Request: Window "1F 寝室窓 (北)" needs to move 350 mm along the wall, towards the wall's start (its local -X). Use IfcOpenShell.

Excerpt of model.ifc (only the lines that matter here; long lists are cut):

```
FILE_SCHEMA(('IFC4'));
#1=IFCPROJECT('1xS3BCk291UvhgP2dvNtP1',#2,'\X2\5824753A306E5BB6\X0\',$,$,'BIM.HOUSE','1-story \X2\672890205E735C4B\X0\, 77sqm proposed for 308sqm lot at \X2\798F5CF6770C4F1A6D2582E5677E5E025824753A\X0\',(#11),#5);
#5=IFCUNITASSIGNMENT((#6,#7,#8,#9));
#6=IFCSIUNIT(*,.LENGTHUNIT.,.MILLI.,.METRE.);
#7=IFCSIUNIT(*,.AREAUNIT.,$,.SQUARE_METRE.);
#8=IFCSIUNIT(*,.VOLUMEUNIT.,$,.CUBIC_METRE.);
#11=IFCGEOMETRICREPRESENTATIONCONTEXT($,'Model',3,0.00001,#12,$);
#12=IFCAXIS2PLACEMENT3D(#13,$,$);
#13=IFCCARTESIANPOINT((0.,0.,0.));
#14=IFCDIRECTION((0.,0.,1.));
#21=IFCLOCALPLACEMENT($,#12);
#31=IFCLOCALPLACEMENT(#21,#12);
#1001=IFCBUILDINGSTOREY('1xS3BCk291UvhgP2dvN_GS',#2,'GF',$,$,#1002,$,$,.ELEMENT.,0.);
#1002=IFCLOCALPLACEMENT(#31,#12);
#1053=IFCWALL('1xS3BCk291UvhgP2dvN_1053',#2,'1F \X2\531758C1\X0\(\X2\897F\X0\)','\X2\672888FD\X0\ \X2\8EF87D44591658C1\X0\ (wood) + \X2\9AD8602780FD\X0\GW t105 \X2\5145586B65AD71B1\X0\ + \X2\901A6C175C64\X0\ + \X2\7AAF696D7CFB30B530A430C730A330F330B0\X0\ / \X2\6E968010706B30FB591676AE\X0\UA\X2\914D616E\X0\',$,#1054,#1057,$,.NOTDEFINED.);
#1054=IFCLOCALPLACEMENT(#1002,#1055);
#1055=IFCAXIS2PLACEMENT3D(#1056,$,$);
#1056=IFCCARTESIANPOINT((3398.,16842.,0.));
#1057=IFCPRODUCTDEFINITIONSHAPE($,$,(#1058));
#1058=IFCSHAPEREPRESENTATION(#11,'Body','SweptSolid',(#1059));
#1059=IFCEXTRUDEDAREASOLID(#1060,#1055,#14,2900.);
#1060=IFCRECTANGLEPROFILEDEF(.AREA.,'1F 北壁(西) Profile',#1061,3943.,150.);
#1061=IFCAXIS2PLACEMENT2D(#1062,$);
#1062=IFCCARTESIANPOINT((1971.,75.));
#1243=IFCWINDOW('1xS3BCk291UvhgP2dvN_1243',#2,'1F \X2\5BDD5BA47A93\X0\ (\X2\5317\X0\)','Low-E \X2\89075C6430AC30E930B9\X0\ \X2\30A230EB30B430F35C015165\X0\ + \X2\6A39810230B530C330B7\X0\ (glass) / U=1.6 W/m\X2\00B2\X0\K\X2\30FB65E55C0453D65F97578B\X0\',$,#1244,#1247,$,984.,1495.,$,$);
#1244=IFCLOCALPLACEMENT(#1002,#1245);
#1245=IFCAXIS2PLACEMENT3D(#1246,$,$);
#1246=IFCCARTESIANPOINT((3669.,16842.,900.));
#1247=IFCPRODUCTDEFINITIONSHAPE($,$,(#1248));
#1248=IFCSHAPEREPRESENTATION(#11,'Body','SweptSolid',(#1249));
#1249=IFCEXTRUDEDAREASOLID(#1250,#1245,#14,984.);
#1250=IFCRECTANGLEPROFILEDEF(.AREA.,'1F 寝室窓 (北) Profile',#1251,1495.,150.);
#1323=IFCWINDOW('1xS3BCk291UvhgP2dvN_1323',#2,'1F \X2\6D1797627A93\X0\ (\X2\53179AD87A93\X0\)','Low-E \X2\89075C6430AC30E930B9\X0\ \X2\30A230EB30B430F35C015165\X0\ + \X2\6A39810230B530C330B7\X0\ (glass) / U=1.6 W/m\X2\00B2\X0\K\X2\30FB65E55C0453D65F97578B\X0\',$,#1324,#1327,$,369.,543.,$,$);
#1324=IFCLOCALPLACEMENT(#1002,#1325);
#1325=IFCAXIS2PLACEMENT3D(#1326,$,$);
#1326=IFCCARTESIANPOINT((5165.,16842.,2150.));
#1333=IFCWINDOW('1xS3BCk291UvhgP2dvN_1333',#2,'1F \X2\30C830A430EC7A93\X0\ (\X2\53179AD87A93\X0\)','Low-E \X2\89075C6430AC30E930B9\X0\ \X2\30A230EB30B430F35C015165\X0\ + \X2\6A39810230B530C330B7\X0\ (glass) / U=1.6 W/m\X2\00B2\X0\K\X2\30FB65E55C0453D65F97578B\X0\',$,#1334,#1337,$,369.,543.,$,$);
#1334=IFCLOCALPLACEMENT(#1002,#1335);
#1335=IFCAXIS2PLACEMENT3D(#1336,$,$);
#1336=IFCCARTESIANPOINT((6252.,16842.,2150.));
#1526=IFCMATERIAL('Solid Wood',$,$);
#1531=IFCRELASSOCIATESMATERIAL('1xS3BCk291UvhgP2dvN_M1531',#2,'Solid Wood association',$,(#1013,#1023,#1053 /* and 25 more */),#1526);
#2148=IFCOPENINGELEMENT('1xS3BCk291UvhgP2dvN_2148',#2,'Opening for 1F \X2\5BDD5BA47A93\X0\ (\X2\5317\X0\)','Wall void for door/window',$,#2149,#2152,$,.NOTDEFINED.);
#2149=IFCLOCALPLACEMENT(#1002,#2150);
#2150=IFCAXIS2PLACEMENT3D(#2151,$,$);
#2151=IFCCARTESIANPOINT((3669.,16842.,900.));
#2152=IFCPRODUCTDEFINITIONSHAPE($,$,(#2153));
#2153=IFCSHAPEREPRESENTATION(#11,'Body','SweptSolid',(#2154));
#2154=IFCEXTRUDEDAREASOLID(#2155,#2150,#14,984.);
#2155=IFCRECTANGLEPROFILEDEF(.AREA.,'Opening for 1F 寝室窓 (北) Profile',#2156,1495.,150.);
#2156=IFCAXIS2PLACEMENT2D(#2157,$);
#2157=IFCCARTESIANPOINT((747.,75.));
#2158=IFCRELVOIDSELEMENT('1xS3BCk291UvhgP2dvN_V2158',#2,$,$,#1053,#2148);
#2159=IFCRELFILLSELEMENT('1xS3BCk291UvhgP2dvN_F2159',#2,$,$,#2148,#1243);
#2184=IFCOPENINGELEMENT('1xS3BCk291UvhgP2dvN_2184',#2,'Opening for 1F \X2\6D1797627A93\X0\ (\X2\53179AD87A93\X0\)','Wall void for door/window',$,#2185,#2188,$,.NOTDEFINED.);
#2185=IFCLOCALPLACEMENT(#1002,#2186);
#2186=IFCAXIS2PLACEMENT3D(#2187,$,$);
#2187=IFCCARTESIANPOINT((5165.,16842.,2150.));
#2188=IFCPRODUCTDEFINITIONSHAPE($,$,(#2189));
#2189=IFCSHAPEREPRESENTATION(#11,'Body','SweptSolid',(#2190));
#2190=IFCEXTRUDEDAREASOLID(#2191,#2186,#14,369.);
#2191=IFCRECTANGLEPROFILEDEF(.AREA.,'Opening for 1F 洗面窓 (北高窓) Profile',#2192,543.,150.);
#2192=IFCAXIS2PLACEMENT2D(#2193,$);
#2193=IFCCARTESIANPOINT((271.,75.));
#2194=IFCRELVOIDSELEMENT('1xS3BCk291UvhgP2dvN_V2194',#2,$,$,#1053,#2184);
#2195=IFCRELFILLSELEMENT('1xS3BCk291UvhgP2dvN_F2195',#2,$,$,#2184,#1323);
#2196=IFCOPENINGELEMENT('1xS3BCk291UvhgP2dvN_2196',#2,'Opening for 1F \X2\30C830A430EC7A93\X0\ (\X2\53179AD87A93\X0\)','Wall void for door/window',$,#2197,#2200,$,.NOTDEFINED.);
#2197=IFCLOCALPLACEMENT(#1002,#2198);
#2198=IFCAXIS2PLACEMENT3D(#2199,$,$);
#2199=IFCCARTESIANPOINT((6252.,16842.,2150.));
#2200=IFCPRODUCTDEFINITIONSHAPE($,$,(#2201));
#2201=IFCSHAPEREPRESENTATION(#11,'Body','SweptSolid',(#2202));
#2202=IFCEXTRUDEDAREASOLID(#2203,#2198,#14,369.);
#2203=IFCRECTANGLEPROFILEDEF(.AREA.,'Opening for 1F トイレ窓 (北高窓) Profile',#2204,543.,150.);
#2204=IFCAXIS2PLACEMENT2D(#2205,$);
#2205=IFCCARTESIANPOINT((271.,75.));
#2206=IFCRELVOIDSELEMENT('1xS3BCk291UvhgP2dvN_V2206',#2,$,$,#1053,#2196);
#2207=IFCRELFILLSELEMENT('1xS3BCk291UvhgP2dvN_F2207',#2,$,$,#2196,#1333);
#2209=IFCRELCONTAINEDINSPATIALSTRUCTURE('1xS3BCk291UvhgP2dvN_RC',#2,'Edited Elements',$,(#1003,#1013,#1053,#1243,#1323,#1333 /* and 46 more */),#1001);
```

```python
import ifcopenshell
import ifcopenshell.api.geometry
import ifcopenshell.util.placement
import ifcopenshell.util.unit

model = ifcopenshell.open("model.ifc")
unit_scale = ifcopenshell.util.unit.calculate_unit_scale(model)

window = model.by_id(1243)
opening = window.FillsVoids[0].RelatingOpeningElement
wall = opening.VoidsElements[0].RelatingBuildingElement

wall_matrix = ifcopenshell.util.placement.get_local_placement(wall.ObjectPlacement)
shift = wall_matrix[:3, 0] * -0.35 / unit_scale
before = ifcopenshell.util.placement.get_local_placement(window.ObjectPlacement)[:3, 3].copy()

# The window is not placed relative to its opening, so move both.
for product in (opening, window):
    matrix = ifcopenshell.util.placement.get_local_placement(product.ObjectPlacement)
    matrix[:3, 3] += shift
    ifcopenshell.api.geometry.edit_object_placement(model, product=product, matrix=matrix, is_si=False)

after = ifcopenshell.util.placement.get_local_placement(window.ObjectPlacement)[:3, 3]
print("window moved by", (after - before).round(3) + 0.0)

model.write("model_rev.ifc")
```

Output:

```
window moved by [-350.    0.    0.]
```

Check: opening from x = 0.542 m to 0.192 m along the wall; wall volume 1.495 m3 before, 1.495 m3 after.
